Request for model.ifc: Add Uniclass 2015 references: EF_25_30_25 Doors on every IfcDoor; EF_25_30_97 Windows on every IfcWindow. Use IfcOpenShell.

First a look at what the model holds.

```python
import ifcopenshell

model = ifcopenshell.open("model.ifc")
print(model.schema)
print("classifications:", [c.Name for c in model.by_type("IfcClassification")])
for ifc_class in ("IfcDoor", "IfcRoof", "IfcStair", "IfcWall", "IfcWindow"):
    print(ifc_class, len(model.by_type(ifc_class)))
```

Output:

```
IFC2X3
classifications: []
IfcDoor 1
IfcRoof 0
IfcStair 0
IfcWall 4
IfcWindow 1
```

```python
import ifcopenshell
import ifcopenshell.api.classification

model = ifcopenshell.open("model.ifc")

# IFC2X3 requires Source and Edition and has no link from the project to the system.
system = model.create_entity("IfcClassification", Source="NBS", Edition="2015", Name="Uniclass 2015")

codes = {
    "IfcDoor": ("EF_25_30_25", "Doors"),
    "IfcWindow": ("EF_25_30_97", "Windows"),
}
for ifc_class, (code, name) in codes.items():
    products = model.by_type(ifc_class)
    ifcopenshell.api.classification.add_reference(
        model, products=products, classification=system, identification=code, name=name
    )
    print(code, len(products))

model.write("model_updated.ifc")
```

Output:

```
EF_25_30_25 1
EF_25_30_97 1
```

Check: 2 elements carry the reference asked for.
